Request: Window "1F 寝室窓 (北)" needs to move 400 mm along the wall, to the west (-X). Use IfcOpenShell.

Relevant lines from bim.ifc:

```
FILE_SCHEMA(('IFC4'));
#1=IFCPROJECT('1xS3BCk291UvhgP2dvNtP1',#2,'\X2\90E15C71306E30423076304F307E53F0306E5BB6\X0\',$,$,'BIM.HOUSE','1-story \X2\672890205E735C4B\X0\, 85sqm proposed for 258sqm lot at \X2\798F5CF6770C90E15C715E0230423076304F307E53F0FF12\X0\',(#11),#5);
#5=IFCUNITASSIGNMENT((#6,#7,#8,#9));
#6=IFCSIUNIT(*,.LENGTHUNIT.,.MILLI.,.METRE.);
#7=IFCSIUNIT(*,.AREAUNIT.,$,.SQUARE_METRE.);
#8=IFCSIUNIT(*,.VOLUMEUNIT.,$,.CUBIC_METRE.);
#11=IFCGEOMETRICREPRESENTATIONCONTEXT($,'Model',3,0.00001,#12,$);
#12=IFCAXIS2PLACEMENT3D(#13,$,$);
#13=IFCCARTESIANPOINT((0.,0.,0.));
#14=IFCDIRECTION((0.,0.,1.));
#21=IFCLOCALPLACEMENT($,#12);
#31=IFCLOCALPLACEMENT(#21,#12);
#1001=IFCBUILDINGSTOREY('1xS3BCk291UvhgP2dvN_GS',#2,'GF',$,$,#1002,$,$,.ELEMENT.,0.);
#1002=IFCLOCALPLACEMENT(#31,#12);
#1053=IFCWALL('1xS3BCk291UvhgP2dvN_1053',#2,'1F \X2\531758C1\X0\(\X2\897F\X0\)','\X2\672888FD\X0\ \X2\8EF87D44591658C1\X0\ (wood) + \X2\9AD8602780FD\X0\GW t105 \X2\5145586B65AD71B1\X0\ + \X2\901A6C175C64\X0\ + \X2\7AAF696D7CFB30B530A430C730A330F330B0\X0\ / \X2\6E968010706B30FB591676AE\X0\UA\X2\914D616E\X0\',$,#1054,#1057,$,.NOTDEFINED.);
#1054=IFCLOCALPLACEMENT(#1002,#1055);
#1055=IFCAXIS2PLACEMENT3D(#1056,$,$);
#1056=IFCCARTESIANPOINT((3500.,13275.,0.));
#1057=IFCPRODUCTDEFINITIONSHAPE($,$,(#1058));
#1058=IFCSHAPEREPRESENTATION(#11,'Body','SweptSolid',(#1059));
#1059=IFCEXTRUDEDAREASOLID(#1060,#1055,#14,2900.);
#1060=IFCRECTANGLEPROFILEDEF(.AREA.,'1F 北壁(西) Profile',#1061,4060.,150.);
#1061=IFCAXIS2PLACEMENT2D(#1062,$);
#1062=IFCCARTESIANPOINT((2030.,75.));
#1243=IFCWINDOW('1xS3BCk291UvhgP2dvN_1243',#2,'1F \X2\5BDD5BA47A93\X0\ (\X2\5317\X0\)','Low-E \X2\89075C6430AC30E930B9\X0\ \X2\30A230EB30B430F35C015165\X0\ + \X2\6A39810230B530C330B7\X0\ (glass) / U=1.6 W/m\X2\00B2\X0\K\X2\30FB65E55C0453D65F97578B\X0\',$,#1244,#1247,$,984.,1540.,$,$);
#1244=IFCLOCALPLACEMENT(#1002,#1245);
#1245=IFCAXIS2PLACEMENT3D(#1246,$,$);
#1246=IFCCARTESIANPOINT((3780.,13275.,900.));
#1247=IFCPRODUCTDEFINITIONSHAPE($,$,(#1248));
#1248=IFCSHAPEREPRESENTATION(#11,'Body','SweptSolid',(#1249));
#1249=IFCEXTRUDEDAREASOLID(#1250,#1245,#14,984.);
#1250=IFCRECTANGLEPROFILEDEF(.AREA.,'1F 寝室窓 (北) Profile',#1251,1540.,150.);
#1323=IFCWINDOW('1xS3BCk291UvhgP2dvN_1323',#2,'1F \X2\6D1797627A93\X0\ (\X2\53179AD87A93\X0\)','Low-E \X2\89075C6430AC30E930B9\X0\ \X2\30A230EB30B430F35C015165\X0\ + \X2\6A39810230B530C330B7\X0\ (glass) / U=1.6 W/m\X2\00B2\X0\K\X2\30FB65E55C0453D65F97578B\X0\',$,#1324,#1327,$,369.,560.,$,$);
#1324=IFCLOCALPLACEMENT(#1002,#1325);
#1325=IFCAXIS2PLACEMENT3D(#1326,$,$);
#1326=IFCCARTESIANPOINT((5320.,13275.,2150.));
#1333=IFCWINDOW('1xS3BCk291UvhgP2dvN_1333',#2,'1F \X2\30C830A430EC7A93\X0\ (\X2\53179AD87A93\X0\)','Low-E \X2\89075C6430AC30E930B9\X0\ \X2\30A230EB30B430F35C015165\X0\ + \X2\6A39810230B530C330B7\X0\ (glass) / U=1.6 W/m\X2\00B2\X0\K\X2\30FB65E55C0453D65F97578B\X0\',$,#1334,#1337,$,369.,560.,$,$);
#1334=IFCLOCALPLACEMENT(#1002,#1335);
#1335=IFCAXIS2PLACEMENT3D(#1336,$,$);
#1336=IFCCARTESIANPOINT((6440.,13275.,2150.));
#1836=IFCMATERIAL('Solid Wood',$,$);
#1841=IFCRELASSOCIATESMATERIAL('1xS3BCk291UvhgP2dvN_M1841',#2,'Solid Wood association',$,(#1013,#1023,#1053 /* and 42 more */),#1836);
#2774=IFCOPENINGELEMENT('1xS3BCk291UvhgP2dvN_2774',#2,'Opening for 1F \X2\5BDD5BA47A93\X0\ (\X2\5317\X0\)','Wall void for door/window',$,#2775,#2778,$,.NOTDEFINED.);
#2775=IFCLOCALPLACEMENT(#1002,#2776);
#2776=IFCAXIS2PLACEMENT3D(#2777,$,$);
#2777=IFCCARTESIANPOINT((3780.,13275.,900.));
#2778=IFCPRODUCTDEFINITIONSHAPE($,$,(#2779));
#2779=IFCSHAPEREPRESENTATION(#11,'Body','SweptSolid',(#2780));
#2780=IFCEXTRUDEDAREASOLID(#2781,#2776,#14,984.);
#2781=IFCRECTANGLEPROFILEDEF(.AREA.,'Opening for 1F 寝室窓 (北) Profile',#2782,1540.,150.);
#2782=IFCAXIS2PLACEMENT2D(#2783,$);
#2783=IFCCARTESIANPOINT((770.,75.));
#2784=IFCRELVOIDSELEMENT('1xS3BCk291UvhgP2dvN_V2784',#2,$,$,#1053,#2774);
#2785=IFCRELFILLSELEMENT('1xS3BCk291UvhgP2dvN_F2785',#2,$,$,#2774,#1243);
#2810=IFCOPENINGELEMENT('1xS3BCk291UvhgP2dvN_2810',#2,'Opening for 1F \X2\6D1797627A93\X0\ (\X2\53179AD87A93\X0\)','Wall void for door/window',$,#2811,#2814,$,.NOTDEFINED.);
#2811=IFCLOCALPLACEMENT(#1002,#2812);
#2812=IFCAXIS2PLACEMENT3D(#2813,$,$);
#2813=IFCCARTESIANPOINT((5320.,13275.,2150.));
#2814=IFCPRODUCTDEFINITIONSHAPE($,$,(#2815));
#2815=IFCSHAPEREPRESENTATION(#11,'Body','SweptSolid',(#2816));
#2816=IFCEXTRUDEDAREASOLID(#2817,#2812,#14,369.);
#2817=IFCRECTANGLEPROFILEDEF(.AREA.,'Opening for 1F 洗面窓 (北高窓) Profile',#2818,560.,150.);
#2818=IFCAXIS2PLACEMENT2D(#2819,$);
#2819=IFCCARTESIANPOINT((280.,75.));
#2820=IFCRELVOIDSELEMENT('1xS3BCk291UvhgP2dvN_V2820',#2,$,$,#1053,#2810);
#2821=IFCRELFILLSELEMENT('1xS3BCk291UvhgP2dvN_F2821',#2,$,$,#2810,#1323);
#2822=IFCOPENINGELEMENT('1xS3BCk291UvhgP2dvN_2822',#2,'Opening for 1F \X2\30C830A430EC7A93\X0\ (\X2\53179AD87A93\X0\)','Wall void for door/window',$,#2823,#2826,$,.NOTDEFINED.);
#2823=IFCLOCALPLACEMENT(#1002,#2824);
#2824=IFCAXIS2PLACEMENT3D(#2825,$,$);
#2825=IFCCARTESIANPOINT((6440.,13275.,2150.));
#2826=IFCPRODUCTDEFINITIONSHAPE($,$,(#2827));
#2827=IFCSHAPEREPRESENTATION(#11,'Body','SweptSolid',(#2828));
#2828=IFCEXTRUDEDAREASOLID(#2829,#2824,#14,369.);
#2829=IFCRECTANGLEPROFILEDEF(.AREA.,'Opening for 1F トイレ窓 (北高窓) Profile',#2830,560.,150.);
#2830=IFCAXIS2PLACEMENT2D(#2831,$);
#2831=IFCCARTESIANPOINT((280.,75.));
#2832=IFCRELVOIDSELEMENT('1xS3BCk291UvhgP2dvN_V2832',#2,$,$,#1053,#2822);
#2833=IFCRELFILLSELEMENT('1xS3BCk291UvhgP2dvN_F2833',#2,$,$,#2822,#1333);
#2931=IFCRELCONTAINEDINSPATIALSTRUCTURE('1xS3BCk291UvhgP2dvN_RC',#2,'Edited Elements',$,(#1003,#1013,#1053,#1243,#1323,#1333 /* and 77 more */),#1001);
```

```python
import ifcopenshell
import ifcopenshell.api.geometry
import ifcopenshell.util.placement

model = ifcopenshell.open("bim.ifc")

window = model.by_guid("1xS3BCk291UvhgP2dvN_1243")
opening = window.FillsVoids[0].RelatingOpeningElement
wall = opening.VoidsElements[0].RelatingBuildingElement

wall_matrix = ifcopenshell.util.placement.get_local_placement(wall.ObjectPlacement)
shift = wall_matrix[:3, 0] * -400.0
before = ifcopenshell.util.placement.get_local_placement(window.ObjectPlacement)[:3, 3].copy()

# The window is not placed relative to its opening, so move both.
for product in (opening, window):
    matrix = ifcopenshell.util.placement.get_local_placement(product.ObjectPlacement)
    matrix[:3, 3] += shift
    ifcopenshell.api.geometry.edit_object_placement(model, product=product, matrix=matrix, is_si=False)

after = ifcopenshell.util.placement.get_local_placement(window.ObjectPlacement)[:3, 3]
print("window moved by", (after - before).round(3) + 0.0)

model.write("bim_rev.ifc")
```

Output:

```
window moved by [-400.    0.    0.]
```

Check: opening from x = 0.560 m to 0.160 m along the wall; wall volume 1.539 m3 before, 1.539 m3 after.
